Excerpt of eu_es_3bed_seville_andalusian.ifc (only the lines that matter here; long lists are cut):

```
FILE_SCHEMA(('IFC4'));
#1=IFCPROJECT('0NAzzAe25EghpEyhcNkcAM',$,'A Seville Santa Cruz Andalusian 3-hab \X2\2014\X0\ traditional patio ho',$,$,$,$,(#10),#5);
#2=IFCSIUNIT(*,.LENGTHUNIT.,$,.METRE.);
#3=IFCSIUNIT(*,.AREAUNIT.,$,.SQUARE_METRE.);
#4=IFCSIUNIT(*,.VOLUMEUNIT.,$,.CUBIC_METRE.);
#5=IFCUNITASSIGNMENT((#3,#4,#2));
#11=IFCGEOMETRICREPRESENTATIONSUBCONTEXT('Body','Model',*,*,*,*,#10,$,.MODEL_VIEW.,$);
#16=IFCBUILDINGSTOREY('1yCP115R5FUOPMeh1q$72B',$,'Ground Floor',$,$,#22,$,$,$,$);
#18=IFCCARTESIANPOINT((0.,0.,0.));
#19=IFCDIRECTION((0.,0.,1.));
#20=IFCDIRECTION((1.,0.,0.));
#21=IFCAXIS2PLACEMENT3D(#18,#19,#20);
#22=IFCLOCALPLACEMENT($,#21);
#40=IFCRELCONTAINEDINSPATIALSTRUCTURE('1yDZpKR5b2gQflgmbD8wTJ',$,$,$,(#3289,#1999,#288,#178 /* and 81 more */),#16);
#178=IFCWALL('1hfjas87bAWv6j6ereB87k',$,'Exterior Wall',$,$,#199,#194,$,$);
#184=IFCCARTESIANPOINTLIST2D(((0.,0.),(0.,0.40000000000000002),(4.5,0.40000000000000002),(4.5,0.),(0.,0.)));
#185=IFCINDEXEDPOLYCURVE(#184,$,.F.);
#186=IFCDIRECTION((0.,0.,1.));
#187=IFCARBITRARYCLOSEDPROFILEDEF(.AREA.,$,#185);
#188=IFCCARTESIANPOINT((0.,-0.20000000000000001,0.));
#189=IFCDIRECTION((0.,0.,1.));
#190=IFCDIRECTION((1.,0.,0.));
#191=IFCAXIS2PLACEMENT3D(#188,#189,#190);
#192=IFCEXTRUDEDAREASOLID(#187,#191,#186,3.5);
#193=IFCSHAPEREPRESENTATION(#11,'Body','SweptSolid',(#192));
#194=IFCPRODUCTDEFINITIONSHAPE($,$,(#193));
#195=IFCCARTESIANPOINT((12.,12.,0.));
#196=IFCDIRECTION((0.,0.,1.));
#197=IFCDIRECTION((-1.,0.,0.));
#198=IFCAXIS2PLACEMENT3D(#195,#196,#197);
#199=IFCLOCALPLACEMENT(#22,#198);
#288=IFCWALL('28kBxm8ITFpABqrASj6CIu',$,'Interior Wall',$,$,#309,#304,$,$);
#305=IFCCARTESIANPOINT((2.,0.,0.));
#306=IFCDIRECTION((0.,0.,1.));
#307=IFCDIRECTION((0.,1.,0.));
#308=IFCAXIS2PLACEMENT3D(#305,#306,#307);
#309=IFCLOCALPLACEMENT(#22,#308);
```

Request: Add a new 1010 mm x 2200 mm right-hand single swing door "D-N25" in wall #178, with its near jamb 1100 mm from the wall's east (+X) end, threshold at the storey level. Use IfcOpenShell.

```python
import numpy as np
import ifcopenshell
import ifcopenshell.api.feature
import ifcopenshell.api.geometry
import ifcopenshell.api.root
import ifcopenshell.api.spatial
import ifcopenshell.geom
import ifcopenshell.util.element
import ifcopenshell.util.placement
import ifcopenshell.util.representation
import ifcopenshell.util.shape
import ifcopenshell.util.unit

model = ifcopenshell.open("eu_es_3bed_seville_andalusian.ifc")
unit_scale = ifcopenshell.util.unit.calculate_unit_scale(model)
settings = ifcopenshell.geom.settings()


def volume(element):
    """Net volume in cubic metres, openings subtracted."""
    shape = ifcopenshell.geom.create_shape(settings, element)
    return ifcopenshell.util.shape.get_volume(shape.geometry)


wall = model.by_guid("1hfjas87bAWv6j6ereB87k")
storey = ifcopenshell.util.element.get_container(wall, ifc_class="IfcBuildingStorey")
context = ifcopenshell.util.representation.get_context(model, "Model", "Body", "MODEL_VIEW")
before = volume(wall)

width, height, from_end, sill = 1.01, 2.2, 1.1, 0.0  # metres

# The wall runs along its own X axis, and the end named is its -X end.
wall_shape = ifcopenshell.geom.create_shape(settings, wall)
x, y, z = ifcopenshell.util.shape.get_vertices(wall_shape.geometry).T
start = x.min() + from_end
face, thickness = float(y.min()), float(y.max() - y.min())
wall_matrix = ifcopenshell.util.placement.get_local_placement(wall.ObjectPlacement)
level = ifcopenshell.util.placement.get_local_placement(storey.ObjectPlacement)[2, 3]


def in_wall(x, y):
    """Placement at x, y metres in the wall's axes, at sill height."""
    matrix = wall_matrix.copy()
    matrix[:, 3] = wall_matrix @ np.array([x / unit_scale, y / unit_scale, 0.0, 1.0])
    matrix[2, 3] = level + sill / unit_scale
    return matrix


# Opening: a box that overshoots both wall faces by 50 mm.
opening = ifcopenshell.api.root.create_entity(model, ifc_class="IfcOpeningElement", predefined_type="OPENING")
box = ifcopenshell.api.geometry.add_wall_representation(
    model, context=context, length=width, height=height, thickness=thickness + 0.1
)
ifcopenshell.api.geometry.assign_representation(model, product=opening, representation=box)
ifcopenshell.api.geometry.edit_object_placement(model, product=opening, matrix=in_wall(start, face - 0.05), is_si=False)
ifcopenshell.api.feature.add_feature(model, feature=opening, element=wall)

door = ifcopenshell.api.root.create_entity(model, ifc_class="IfcDoor", name="D-N25", predefined_type="DOOR")
door.OverallWidth, door.OverallHeight = width / unit_scale, height / unit_scale
door.OperationType = "SINGLE_SWING_RIGHT"
body = ifcopenshell.api.geometry.add_door_representation(
    model,
    context=context,
    overall_width=door.OverallWidth,
    overall_height=door.OverallHeight,
    operation_type="SINGLE_SWING_RIGHT",
    lining_properties={"LiningDepth": thickness / unit_scale, "ThresholdDepth": thickness / unit_scale},
)
ifcopenshell.api.geometry.assign_representation(model, product=door, representation=body)
ifcopenshell.api.spatial.assign_container(model, products=[door], relating_structure=storey)
ifcopenshell.api.feature.add_filling(model, opening=opening, element=door)

# The lining spans the wall, so the door starts at the wall face.
ifcopenshell.api.geometry.edit_object_placement(model, product=door, matrix=in_wall(start, face), is_si=False)

after = volume(wall)

print(f"wall volume {before:.3f} -> {after:.3f} m3")

model.write("eu_es_3bed_seville_andalusian-out.ifc")
```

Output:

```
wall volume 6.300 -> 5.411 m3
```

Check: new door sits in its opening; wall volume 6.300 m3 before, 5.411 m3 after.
